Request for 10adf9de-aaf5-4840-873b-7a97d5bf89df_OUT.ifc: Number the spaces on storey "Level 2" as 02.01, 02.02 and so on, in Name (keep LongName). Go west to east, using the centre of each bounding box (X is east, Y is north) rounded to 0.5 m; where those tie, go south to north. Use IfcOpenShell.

First a look at what the model holds.

```python
import ifcopenshell
import ifcopenshell.util.element
import ifcopenshell.util.placement

model = ifcopenshell.open("10adf9de-aaf5-4840-873b-7a97d5bf89df_OUT.ifc")
print(model.schema)
storey = next(s for s in model.by_type("IfcBuildingStorey") if s.Name == "Level 2")
spaces = [e for e in ifcopenshell.util.element.get_decomposition(storey) if e.is_a("IfcSpace")]
for e in sorted(spaces, key=lambda e: e.id()):
    origin = ifcopenshell.util.placement.get_local_placement(e.ObjectPlacement)[:3, 3]
    print(e.id(), e.Name, e.LongName, origin.round(2) + 0.0, sep=" | ")
```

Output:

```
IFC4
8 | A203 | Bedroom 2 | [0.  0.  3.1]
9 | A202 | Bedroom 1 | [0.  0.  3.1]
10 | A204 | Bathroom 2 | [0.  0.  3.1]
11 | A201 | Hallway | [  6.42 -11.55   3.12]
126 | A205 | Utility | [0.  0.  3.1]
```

```python
import ifcopenshell
import ifcopenshell.geom
import ifcopenshell.util.element
import ifcopenshell.util.shape

model = ifcopenshell.open("10adf9de-aaf5-4840-873b-7a97d5bf89df_OUT.ifc")
settings = ifcopenshell.geom.settings()
settings.set("use-world-coords", True)


def centre(element):
    shape = ifcopenshell.geom.create_shape(settings, element)
    return ifcopenshell.util.shape.get_bbox_centroid(shape.geometry)


storey = next(s for s in model.by_type("IfcBuildingStorey") if s.Name == "Level 2")
spaces = [e for e in ifcopenshell.util.element.get_decomposition(storey) if e.is_a("IfcSpace")]

# Insertion points can sit at a corner or the storey origin, so sort by the geometry (in metres).
centres = {e: centre(e) for e in spaces}
spaces.sort(key=lambda e: (round(centres[e][0] / 0.5), centres[e][1]))

for i, e in enumerate(spaces, start=1):
    number = f"02.{i:02d}"
    e.Name = number
    print(e.id(), number)

model.write("10adf9de-aaf5-4840-873b-7a97d5bf89df_OUT-out.ifc")
```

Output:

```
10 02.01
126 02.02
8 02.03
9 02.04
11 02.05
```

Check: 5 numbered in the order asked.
